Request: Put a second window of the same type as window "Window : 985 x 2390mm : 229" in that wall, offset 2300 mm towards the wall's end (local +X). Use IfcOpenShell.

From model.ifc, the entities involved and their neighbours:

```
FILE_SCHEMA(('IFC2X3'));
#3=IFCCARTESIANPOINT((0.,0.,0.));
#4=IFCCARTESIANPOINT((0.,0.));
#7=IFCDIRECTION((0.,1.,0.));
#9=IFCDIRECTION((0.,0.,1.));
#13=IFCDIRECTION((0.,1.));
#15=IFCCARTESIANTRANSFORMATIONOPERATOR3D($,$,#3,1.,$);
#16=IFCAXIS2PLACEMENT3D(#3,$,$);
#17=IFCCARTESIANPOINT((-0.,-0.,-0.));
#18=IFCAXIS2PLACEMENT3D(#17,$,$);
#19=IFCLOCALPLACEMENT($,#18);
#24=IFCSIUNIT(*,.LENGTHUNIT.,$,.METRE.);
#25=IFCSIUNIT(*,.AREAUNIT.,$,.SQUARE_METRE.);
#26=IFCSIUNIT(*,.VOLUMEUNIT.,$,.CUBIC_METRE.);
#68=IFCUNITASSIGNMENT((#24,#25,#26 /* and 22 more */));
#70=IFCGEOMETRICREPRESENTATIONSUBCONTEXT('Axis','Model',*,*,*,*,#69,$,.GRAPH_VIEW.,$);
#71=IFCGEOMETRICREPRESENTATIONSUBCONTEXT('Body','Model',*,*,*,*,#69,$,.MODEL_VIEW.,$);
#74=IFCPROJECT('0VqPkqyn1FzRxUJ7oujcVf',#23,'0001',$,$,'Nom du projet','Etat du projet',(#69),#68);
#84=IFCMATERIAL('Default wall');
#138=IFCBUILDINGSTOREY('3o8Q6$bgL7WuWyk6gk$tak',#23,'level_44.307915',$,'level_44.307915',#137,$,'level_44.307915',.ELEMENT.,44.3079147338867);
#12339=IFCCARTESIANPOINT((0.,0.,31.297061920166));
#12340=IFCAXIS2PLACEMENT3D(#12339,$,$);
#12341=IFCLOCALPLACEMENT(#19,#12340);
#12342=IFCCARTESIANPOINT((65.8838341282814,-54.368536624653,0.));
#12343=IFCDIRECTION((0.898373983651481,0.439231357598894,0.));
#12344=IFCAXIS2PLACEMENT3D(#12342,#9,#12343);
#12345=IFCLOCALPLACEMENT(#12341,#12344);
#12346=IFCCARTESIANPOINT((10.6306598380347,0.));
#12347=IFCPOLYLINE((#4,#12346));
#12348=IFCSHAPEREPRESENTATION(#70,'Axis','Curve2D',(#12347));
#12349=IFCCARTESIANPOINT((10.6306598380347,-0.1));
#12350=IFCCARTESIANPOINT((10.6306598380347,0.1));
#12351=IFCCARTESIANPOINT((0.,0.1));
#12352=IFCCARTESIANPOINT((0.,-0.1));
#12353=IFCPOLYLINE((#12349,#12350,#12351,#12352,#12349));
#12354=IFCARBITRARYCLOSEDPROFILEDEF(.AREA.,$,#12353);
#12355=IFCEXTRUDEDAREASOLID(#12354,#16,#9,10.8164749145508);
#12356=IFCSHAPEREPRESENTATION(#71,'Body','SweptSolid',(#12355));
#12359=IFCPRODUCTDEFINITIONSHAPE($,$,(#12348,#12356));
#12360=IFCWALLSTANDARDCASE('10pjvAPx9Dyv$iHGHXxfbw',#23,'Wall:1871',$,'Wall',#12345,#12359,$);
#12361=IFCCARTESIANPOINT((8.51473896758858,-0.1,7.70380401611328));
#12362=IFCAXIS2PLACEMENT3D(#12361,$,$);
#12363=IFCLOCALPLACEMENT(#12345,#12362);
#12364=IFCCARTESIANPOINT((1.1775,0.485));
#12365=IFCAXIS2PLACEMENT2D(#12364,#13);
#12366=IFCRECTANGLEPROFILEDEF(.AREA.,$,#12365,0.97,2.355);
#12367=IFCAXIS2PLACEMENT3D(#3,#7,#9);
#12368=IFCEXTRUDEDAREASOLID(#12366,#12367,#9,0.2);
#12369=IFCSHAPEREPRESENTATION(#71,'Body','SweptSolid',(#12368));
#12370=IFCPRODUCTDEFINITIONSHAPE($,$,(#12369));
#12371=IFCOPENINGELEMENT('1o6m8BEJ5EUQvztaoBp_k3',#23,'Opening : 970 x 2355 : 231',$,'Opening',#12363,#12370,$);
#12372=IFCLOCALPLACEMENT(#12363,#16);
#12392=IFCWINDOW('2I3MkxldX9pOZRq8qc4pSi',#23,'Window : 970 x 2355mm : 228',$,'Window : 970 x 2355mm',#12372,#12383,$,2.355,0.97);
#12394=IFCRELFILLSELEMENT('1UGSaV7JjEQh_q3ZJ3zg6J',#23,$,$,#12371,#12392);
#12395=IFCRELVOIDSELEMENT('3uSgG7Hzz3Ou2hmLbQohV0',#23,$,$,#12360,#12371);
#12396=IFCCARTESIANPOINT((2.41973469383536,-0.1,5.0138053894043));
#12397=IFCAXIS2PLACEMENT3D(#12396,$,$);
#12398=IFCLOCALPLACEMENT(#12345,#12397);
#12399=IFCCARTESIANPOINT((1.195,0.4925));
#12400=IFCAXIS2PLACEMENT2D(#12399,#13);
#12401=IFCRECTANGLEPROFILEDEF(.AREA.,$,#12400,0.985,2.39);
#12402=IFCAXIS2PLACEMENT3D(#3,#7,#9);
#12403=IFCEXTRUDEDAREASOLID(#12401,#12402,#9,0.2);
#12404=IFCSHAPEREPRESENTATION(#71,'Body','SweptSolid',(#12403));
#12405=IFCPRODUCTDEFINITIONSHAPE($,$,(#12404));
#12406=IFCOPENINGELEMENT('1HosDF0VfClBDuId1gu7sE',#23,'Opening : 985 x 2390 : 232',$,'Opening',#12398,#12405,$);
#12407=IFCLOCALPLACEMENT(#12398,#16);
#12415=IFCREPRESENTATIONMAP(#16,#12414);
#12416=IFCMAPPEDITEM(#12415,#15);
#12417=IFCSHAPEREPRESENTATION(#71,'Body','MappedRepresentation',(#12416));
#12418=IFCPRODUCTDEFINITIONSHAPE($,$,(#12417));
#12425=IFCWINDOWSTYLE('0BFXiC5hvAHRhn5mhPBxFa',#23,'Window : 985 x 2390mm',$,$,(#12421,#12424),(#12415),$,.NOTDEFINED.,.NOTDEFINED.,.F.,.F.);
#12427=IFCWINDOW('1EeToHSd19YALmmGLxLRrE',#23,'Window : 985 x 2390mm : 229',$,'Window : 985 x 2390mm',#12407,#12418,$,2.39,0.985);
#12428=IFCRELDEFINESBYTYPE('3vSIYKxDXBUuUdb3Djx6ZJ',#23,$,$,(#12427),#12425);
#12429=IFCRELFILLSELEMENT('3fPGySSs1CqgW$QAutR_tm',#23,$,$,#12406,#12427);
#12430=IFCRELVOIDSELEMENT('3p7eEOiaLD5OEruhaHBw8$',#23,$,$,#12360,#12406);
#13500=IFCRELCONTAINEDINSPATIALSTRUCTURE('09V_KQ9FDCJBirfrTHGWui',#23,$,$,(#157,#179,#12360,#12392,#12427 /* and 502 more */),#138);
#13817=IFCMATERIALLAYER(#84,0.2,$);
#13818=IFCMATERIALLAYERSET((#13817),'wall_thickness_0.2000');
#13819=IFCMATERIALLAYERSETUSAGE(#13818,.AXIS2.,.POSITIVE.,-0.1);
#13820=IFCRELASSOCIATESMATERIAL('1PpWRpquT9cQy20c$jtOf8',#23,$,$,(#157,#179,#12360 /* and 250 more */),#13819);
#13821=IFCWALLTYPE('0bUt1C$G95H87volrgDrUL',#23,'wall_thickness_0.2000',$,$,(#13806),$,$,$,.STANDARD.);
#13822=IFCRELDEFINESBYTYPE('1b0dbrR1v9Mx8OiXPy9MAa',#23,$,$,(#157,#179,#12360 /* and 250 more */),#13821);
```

```python
import ifcopenshell
import ifcopenshell.api.feature
import ifcopenshell.api.geometry
import ifcopenshell.api.root
import ifcopenshell.geom
import ifcopenshell.util.element
import ifcopenshell.util.placement
import ifcopenshell.util.shape

model = ifcopenshell.open("model.ifc")
settings = ifcopenshell.geom.settings()


def volume(element):
    """Net volume in cubic metres, openings subtracted."""
    shape = ifcopenshell.geom.create_shape(settings, element)
    return ifcopenshell.util.shape.get_volume(shape.geometry)


window = model.by_id(12427)
opening = window.FillsVoids[0].RelatingOpeningElement
wall = opening.VoidsElements[0].RelatingBuildingElement
before = volume(wall)
shift = ifcopenshell.util.placement.get_local_placement(wall.ObjectPlacement)[:3, 0] * 2.3

# copy_class copies the void relationship, type, container and properties, but no geometry.
new_opening = ifcopenshell.api.root.copy_class(model, product=opening)
new_opening.Representation = ifcopenshell.util.element.copy_deep(
    model, opening.Representation, exclude=["IfcGeometricRepresentationContext", "IfcRepresentationMap"]
)
new_opening.Name = "Opening : 985 x 2390"
new_window = ifcopenshell.api.root.copy_class(model, product=window)
new_window.Representation = ifcopenshell.util.element.copy_deep(
    model, window.Representation, exclude=["IfcGeometricRepresentationContext", "IfcRepresentationMap"]
)
new_window.Name = "Window : 985 x 2390mm"
fills = ifcopenshell.api.feature.add_filling(model, opening=new_opening, element=new_window)
fills.OwnerHistory = new_window.OwnerHistory  # required in IFC2X3

for old, new in ((opening, new_opening), (window, new_window)):
    matrix = ifcopenshell.util.placement.get_local_placement(old.ObjectPlacement)
    matrix[:3, 3] += shift
    ifcopenshell.api.geometry.edit_object_placement(model, product=new, matrix=matrix, is_si=False)

after = volume(wall)

print(f"wall volume {before:.3f} -> {after:.3f} m3")

model.write("model_rev.ifc")
```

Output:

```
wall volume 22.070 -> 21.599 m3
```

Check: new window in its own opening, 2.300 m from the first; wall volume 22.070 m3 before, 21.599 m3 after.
